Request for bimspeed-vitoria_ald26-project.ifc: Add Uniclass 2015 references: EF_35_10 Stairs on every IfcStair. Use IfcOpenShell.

First a look at what the model holds.

```python
import ifcopenshell

model = ifcopenshell.open("bimspeed-vitoria_ald26-project.ifc")
print(model.schema)
print("classifications:", [c.Name for c in model.by_type("IfcClassification")])
for ifc_class in ("IfcDoor", "IfcRoof", "IfcStair", "IfcWall", "IfcWindow"):
    print(ifc_class, len(model.by_type(ifc_class)))
```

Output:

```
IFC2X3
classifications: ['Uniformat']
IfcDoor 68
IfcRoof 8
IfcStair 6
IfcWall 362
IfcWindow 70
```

```python
import ifcopenshell
import ifcopenshell.api.classification

model = ifcopenshell.open("bimspeed-vitoria_ald26-project.ifc")

# IFC2X3 requires Source and Edition and has no link from the project to the system.
system = model.create_entity("IfcClassification", Source="NBS", Edition="2015", Name="Uniclass 2015")

codes = {
    "IfcStair": ("EF_35_10", "Stairs"),
}
for ifc_class, (code, name) in codes.items():
    products = model.by_type(ifc_class)
    ifcopenshell.api.classification.add_reference(
        model, products=products, classification=system, identification=code, name=name
    )
    print(code, len(products))

model.write("bimspeed-vitoria_ald26-project_rev.ifc")
```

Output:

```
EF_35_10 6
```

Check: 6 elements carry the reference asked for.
